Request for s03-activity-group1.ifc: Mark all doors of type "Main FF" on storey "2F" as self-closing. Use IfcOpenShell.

First a look at what the model holds.

```python
import ifcopenshell
import ifcopenshell.util.element

model = ifcopenshell.open("s03-activity-group1.ifc")
print(model.schema)
storey = next(s for s in model.by_type("IfcBuildingStorey") if s.Name == "2F")
doors = [e for e in ifcopenshell.util.element.get_decomposition(storey) if e.is_a("IfcDoor")]
seen = {}
for e in doors:
    element_type = ifcopenshell.util.element.get_type(e)
    key = (element_type.Name if element_type != e and element_type else None, ifcopenshell.util.element.get_pset(e, "Pset_DoorCommon", "SelfClosing"))
    seen[key] = seen.get(key, 0) + 1
for (name, value), count in sorted(seen.items(), key=str):
    print(count, "x", name, "|", value)
```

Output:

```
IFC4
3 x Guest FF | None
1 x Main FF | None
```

```python
import ifcopenshell
import ifcopenshell.api.pset
import ifcopenshell.util.element

model = ifcopenshell.open("s03-activity-group1.ifc")

storey = next(s for s in model.by_type("IfcBuildingStorey") if s.Name == "2F")
doors = [e for e in ifcopenshell.util.element.get_decomposition(storey) if e.is_a("IfcDoor")]

count = 0
for e in doors:
    element_type = ifcopenshell.util.element.get_type(e)
    if element_type in (None, e) or element_type.Name != "Main FF":
        continue
    # add_pset returns the element's existing set when there is one.
    pset = ifcopenshell.api.pset.add_pset(model, product=e, name="Pset_DoorCommon")
    ifcopenshell.api.pset.edit_pset(model, pset=pset, properties={"SelfClosing": True})
    count += 1

print(count, "doors updated")

model.write("s03-activity-group1-out.ifc")
```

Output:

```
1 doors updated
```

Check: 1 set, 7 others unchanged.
